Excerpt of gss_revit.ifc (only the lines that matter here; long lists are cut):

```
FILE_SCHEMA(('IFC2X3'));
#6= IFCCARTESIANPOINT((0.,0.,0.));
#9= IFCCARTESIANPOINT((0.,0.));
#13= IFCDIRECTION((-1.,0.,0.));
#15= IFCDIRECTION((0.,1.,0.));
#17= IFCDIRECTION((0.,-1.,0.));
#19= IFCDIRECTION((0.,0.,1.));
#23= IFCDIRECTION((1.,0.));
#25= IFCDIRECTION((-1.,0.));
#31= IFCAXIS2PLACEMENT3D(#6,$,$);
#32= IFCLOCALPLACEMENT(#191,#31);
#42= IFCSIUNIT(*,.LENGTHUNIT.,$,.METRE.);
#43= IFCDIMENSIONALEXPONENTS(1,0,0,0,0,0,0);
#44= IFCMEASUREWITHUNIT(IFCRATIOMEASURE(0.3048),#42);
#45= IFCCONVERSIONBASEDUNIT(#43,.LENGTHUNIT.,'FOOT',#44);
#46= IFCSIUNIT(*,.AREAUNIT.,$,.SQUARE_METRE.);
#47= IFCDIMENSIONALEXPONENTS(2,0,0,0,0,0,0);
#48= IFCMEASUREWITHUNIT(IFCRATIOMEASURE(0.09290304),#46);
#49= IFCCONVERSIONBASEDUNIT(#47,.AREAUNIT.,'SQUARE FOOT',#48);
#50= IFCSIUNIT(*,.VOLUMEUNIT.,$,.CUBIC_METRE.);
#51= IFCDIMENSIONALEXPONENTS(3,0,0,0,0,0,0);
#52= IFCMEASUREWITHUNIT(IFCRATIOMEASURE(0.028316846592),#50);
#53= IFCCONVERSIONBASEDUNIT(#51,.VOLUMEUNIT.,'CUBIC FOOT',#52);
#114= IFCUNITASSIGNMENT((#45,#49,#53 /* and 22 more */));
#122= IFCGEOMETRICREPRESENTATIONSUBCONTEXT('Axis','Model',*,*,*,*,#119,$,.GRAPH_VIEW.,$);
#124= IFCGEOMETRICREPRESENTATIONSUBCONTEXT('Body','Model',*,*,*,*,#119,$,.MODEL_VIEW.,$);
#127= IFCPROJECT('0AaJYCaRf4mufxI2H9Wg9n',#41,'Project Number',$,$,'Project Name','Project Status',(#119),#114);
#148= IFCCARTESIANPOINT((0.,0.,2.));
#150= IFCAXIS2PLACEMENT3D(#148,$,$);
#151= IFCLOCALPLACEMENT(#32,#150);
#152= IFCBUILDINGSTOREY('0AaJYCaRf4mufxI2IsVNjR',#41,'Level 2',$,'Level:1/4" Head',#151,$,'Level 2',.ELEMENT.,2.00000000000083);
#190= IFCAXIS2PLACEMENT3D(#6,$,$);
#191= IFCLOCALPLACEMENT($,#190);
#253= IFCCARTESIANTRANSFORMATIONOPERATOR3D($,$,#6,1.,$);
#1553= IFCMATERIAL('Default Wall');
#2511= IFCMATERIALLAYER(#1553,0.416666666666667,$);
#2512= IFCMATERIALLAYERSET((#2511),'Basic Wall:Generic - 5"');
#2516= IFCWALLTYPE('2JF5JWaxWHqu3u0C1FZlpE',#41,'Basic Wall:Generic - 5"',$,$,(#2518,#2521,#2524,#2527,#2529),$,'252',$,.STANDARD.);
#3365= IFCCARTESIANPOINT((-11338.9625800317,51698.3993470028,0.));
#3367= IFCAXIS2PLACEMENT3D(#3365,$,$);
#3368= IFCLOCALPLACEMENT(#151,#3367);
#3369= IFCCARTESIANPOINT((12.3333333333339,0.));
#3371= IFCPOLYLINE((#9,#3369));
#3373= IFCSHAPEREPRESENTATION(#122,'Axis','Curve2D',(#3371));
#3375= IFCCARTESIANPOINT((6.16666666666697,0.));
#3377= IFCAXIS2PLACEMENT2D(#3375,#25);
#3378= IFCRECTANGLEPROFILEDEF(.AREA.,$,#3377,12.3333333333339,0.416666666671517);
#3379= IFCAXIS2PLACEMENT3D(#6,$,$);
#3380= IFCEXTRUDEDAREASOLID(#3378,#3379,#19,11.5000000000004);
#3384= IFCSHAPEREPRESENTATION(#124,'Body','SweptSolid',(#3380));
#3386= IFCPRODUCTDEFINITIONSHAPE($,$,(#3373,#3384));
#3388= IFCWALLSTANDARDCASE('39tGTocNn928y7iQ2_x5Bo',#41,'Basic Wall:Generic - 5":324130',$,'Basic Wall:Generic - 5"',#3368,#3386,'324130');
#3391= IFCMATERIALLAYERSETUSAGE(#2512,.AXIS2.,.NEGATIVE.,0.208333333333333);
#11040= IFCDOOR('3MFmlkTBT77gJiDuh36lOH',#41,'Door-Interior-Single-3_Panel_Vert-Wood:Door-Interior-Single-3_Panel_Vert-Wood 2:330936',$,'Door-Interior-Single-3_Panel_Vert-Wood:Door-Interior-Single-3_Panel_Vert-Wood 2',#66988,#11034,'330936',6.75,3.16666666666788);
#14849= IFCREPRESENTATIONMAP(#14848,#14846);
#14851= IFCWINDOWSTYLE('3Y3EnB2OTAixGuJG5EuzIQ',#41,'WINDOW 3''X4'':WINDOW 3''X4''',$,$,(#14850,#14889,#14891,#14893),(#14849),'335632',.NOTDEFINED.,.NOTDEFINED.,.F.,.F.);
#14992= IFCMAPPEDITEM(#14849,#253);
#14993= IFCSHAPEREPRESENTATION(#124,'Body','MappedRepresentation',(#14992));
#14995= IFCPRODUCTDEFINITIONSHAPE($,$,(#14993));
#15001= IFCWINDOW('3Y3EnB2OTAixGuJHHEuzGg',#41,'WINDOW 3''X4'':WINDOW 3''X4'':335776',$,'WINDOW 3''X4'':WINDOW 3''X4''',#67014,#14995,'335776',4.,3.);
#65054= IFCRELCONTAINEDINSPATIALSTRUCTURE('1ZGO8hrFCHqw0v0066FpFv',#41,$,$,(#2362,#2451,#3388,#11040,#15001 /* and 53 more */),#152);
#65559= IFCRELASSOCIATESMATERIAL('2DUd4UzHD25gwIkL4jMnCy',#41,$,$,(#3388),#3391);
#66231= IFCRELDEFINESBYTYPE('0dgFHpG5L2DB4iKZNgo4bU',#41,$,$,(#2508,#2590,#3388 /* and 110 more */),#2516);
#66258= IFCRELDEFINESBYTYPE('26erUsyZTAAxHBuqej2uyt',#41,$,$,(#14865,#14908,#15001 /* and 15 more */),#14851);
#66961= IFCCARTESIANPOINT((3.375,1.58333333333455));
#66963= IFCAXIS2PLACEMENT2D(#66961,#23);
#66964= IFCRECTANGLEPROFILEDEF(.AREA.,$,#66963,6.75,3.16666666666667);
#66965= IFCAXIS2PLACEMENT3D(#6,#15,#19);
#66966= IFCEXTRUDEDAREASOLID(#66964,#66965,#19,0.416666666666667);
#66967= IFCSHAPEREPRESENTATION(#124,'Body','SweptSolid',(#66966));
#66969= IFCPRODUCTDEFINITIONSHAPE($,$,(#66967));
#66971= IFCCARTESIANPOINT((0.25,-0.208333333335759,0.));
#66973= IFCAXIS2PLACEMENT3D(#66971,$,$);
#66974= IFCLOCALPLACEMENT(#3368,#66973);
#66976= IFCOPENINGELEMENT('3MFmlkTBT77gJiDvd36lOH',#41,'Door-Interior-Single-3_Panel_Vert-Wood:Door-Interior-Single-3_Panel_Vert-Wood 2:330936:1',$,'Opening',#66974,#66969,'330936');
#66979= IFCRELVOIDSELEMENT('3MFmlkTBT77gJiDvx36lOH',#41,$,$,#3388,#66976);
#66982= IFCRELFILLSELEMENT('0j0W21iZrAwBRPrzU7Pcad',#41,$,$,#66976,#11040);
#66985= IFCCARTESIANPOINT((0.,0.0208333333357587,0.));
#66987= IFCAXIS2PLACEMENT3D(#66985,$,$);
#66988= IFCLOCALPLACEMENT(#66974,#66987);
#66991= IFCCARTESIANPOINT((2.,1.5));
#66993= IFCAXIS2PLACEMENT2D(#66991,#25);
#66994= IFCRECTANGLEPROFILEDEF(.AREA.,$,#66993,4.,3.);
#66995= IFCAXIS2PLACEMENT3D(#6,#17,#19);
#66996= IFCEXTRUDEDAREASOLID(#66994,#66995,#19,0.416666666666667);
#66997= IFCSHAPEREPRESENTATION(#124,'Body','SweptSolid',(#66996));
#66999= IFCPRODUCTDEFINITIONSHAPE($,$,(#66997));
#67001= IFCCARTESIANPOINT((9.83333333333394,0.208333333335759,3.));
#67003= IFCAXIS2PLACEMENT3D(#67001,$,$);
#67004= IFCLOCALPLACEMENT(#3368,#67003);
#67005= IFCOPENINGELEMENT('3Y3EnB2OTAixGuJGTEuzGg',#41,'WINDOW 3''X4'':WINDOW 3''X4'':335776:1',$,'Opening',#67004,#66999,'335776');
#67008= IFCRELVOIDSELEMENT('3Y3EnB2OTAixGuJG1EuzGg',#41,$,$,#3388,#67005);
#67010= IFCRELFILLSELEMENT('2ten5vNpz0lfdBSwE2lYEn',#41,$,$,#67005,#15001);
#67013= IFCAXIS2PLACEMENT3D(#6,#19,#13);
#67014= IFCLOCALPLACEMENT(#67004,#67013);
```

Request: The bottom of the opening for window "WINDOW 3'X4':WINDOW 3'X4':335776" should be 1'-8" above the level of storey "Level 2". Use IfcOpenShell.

```python
import numpy as np
import ifcopenshell
import ifcopenshell.api.geometry
import ifcopenshell.geom
import ifcopenshell.util.element
import ifcopenshell.util.placement
import ifcopenshell.util.shape
import ifcopenshell.util.unit

model = ifcopenshell.open("gss_revit.ifc")
unit_scale = ifcopenshell.util.unit.calculate_unit_scale(model)

window = model.by_guid("3Y3EnB2OTAixGuJHHEuzGg")
opening = window.FillsVoids[0].RelatingOpeningElement
storey = ifcopenshell.util.element.get_container(window, ifc_class="IfcBuildingStorey")
level = ifcopenshell.util.placement.get_local_placement(storey.ObjectPlacement)[2, 3]

# The opening's origin need not be at the sill, so measure its lowest point.
shape = ifcopenshell.geom.create_shape(ifcopenshell.geom.settings(), opening)
bottom = ifcopenshell.util.shape.get_shape_bottom_elevation(shape, shape.geometry) / unit_scale
dz = level + 20 * 0.0254 / unit_scale - bottom

shift = np.array([0.0, 0.0, dz])
# The window is placed relative to its opening, so it follows when the opening moves.
matrix = ifcopenshell.util.placement.get_local_placement(opening.ObjectPlacement)
matrix[:3, 3] += shift
ifcopenshell.api.geometry.edit_object_placement(
    model, product=opening, matrix=matrix, is_si=False, should_transform_children=True
)

print(f"moved by {dz * unit_scale:+.3f} m")

model.write("gss_revit_rev.ifc")
```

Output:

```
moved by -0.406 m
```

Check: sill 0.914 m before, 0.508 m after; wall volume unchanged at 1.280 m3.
